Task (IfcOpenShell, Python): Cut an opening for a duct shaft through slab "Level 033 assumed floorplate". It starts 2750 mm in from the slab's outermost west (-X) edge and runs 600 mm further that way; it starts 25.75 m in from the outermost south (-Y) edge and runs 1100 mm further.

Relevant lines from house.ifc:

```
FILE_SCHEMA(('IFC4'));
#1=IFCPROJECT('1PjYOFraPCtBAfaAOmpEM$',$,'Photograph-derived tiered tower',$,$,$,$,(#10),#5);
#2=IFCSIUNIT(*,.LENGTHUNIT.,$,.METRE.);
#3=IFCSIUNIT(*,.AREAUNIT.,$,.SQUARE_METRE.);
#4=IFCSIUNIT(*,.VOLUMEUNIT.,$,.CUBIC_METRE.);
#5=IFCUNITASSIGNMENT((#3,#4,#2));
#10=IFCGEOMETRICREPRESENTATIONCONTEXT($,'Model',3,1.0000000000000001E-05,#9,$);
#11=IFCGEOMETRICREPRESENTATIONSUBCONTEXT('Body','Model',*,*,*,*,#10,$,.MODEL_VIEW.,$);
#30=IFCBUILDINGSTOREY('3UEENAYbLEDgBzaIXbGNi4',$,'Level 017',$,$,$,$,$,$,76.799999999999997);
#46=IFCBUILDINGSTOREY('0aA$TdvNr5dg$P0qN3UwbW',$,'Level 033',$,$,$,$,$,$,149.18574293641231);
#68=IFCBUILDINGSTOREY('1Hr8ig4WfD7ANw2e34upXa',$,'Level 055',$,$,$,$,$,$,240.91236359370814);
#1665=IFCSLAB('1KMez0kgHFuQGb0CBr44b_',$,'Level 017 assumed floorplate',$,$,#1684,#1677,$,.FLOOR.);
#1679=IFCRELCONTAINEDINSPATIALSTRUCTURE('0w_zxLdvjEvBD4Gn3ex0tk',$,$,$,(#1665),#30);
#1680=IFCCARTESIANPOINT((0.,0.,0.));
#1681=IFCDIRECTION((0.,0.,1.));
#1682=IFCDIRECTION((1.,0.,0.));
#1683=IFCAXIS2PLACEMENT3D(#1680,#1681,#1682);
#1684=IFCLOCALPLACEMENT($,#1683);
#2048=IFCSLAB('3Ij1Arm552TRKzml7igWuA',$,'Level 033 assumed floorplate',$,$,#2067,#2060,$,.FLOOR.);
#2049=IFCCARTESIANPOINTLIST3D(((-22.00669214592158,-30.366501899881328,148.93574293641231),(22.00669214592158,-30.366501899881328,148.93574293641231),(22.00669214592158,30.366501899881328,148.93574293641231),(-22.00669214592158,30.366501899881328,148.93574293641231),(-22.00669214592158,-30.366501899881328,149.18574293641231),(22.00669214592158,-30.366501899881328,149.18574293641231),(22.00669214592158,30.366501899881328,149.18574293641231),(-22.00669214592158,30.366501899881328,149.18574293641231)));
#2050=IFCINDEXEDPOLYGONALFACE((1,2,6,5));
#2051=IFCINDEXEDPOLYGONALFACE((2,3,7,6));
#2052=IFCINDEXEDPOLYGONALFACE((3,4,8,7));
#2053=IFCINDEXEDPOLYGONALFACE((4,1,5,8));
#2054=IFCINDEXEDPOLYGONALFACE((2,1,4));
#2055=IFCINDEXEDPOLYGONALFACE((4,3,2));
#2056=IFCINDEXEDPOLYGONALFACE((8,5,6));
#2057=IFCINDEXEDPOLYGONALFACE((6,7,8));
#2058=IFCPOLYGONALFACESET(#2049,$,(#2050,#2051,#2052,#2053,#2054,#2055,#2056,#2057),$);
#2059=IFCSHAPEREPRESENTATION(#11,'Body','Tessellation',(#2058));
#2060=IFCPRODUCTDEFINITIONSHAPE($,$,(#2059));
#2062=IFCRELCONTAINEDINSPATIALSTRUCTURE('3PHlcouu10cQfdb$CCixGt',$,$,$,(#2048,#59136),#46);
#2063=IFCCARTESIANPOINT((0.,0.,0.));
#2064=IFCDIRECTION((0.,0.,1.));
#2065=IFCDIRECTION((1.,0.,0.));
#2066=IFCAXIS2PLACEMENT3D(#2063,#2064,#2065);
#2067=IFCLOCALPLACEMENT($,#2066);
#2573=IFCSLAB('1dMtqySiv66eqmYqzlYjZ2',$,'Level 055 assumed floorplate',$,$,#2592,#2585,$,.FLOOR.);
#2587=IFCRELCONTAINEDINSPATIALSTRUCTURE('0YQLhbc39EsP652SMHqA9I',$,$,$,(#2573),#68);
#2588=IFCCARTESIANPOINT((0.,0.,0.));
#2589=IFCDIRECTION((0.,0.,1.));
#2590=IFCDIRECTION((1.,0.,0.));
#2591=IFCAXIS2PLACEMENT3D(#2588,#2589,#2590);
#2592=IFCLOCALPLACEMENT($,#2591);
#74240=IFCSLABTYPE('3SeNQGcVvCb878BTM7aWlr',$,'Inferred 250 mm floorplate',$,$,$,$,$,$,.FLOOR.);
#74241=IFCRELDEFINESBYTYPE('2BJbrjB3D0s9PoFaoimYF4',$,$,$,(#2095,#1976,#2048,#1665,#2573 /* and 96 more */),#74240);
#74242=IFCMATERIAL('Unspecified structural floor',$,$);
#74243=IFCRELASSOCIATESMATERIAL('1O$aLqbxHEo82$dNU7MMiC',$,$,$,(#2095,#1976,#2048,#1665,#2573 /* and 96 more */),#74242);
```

```python
import numpy as np
import ifcopenshell
import ifcopenshell.api.feature
import ifcopenshell.api.geometry
import ifcopenshell.api.root
import ifcopenshell.geom
import ifcopenshell.util.placement
import ifcopenshell.util.representation
import ifcopenshell.util.shape
import ifcopenshell.util.unit

model = ifcopenshell.open("house.ifc")
unit_scale = ifcopenshell.util.unit.calculate_unit_scale(model)
settings = ifcopenshell.geom.settings()


def volume(element):
    """Net volume in cubic metres, openings subtracted."""
    shape = ifcopenshell.geom.create_shape(settings, element)
    return ifcopenshell.util.shape.get_volume(shape.geometry)


slab = model.by_guid("3Ij1Arm552TRKzml7igWuA")
before = volume(slab)

# Extent in the slab's own axes, in metres. The edges named are its -X and -Y sides.
slab_shape = ifcopenshell.geom.create_shape(settings, slab)
vertices = ifcopenshell.util.shape.get_vertices(slab_shape.geometry)
x_min, y_min, bottom = vertices.min(axis=0)
top = vertices[:, 2].max()

opening = ifcopenshell.api.root.create_entity(model, ifc_class="IfcOpeningElement", name="Duct shaft opening", predefined_type="OPENING")
context = ifcopenshell.util.representation.get_context(model, "Model", "Body", "MODEL_VIEW")
width, depth = 0.6, 1.1
outline = [(0.0, 0.0), (width, 0.0), (width, depth), (0.0, depth), (0.0, 0.0)]
# Overshoot both faces by 50 mm so the cut is clean.
shape = ifcopenshell.api.geometry.add_slab_representation(
    model, context=context, depth=top - bottom + 0.1, polyline=outline
)
ifcopenshell.api.geometry.assign_representation(model, product=opening, representation=shape)

matrix = ifcopenshell.util.placement.get_local_placement(slab.ObjectPlacement)
matrix[:, 3] = matrix @ np.append(np.array([x_min + 2.75, y_min + 25.75, bottom - 0.05]) / unit_scale, 1.0)
ifcopenshell.api.geometry.edit_object_placement(model, product=opening, matrix=matrix, is_si=False)
ifcopenshell.api.feature.add_feature(model, feature=opening, element=slab)

after = volume(slab)

print(f"slab volume {before:.3f} -> {after:.3f} m3")

model.write("house_v2.ifc")
```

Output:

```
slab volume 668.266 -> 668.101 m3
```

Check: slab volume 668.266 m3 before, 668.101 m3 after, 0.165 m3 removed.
